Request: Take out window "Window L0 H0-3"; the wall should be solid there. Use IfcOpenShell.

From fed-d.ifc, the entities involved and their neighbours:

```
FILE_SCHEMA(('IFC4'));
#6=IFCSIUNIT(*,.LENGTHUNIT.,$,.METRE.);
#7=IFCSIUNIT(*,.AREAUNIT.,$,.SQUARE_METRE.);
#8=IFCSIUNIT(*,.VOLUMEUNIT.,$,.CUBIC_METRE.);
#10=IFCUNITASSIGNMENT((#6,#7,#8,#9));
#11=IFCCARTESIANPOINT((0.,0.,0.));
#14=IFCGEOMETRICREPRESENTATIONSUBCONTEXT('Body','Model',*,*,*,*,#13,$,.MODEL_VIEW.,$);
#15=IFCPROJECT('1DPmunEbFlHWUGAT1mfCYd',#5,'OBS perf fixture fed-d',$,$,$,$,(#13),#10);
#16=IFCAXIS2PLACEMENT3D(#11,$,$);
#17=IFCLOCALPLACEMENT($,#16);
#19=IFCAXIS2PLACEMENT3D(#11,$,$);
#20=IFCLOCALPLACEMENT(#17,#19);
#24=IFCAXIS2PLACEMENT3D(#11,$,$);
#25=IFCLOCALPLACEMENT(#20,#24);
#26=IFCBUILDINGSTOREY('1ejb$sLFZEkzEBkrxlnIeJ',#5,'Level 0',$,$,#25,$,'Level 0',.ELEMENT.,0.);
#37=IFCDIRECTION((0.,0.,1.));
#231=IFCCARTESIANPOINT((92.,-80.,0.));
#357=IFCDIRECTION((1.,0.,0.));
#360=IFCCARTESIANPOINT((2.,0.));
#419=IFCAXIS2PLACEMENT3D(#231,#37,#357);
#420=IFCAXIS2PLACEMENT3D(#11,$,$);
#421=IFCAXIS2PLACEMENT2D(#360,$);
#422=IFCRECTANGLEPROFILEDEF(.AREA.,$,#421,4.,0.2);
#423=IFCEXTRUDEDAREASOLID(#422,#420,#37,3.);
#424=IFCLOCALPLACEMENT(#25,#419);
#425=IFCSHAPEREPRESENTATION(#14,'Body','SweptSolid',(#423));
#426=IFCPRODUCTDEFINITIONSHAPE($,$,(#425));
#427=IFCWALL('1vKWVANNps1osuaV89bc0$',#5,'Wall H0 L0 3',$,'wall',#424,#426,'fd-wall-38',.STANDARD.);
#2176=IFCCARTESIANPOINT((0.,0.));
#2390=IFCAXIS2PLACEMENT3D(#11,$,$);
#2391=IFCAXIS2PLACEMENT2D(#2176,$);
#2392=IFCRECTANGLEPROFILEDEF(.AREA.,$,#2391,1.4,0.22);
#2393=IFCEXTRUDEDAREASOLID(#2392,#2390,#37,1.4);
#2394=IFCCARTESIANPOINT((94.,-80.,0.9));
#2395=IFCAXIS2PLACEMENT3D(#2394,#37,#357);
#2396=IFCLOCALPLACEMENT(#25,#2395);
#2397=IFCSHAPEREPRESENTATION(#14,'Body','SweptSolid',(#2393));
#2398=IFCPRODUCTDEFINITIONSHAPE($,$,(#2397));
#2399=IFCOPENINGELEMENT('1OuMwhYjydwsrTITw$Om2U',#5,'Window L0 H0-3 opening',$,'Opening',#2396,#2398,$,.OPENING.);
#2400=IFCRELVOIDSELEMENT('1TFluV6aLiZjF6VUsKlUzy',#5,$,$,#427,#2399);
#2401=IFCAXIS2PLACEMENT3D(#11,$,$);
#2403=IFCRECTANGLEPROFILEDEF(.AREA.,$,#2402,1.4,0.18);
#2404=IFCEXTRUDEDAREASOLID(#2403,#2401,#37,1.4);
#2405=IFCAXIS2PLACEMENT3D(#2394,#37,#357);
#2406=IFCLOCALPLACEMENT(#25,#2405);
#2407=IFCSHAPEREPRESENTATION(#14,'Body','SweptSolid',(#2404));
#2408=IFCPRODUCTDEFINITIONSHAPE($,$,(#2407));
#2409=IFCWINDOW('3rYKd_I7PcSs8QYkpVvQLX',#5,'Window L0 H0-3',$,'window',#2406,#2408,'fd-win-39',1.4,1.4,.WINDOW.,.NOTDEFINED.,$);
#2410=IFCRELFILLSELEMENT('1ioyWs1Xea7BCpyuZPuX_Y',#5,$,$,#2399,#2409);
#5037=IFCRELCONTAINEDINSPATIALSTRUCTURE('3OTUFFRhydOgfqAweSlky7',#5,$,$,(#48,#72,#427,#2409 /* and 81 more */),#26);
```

```python
import ifcopenshell
import ifcopenshell.api.feature
import ifcopenshell.api.root
import ifcopenshell.geom
import ifcopenshell.util.shape

model = ifcopenshell.open("fed-d.ifc")
settings = ifcopenshell.geom.settings()


def volume(element):
    """Net volume in cubic metres, openings subtracted."""
    shape = ifcopenshell.geom.create_shape(settings, element)
    return ifcopenshell.util.shape.get_volume(shape.geometry)


window = model.by_id(2409)
opening = window.FillsVoids[0].RelatingOpeningElement
wall = opening.VoidsElements[0].RelatingBuildingElement
before = volume(wall)

ifcopenshell.api.root.remove_product(model, product=window)
ifcopenshell.api.feature.remove_feature(model, feature=opening)

after = volume(wall)

print(f"wall volume {before:.3f} -> {after:.3f} m3")

model.write("fed-d_edited.ifc")
```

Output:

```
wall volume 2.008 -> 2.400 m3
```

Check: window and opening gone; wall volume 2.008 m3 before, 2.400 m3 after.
